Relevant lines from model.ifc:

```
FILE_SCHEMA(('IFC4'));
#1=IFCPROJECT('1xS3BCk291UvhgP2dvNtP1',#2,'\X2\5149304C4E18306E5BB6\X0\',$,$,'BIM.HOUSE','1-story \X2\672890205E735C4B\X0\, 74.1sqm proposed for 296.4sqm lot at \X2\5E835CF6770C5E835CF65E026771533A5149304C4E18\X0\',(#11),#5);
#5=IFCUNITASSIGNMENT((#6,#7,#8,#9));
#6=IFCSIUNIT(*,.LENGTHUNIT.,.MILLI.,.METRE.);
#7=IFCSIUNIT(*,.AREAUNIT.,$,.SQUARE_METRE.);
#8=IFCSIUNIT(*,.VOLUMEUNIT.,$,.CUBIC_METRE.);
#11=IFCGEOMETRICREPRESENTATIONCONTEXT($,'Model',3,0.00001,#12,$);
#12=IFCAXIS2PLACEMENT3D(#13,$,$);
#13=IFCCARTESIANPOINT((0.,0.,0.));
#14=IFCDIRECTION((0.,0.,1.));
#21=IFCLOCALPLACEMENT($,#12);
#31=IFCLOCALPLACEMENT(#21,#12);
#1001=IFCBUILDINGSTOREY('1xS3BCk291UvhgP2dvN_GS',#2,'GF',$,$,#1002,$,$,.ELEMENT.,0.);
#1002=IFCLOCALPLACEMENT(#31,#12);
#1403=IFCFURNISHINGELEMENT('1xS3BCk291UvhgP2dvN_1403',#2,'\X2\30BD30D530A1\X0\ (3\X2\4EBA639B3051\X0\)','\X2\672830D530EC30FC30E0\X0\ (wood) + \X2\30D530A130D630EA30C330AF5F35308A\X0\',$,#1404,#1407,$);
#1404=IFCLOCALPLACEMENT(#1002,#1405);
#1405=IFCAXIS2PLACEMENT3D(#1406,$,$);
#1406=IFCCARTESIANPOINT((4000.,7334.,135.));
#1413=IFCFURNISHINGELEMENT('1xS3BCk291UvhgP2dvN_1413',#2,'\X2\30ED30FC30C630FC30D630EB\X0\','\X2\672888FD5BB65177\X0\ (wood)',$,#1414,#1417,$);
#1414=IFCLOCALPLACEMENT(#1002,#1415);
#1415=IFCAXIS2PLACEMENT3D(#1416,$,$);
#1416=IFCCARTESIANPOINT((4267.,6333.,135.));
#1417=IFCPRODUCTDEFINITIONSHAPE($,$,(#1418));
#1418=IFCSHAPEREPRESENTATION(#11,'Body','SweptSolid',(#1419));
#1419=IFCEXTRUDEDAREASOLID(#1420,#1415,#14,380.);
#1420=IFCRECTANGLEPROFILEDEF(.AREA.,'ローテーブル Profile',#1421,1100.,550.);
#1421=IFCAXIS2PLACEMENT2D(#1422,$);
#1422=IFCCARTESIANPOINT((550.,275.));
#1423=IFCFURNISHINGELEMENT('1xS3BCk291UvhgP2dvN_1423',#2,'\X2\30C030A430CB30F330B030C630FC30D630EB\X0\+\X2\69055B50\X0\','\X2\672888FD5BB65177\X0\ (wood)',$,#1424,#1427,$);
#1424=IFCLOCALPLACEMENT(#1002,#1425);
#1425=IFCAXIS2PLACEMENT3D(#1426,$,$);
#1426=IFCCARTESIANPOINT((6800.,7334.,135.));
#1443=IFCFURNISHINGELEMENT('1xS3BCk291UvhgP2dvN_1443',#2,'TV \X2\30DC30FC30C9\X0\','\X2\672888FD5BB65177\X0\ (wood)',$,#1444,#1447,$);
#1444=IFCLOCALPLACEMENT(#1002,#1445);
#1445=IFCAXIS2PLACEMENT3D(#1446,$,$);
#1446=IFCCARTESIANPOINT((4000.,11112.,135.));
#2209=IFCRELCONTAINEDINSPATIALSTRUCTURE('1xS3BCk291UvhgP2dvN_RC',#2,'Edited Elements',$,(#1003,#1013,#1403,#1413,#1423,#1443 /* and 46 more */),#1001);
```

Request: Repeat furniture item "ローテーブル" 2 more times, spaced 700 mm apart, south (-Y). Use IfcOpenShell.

```python
import numpy as np
import ifcopenshell
import ifcopenshell.api.geometry
import ifcopenshell.api.root
import ifcopenshell.util.element
import ifcopenshell.util.placement
import ifcopenshell.util.unit

model = ifcopenshell.open("model.ifc")
unit_scale = ifcopenshell.util.unit.calculate_unit_scale(model)


def reuse_history(source, copy):
    """copy_class also copies each property set's owner history, people and application; keep the originals."""
    for rel in copy.IsDefinedBy:
        if rel.is_a("IfcRelDefinesByProperties") and (history := rel.RelatingPropertyDefinition.OwnerHistory):
            rel.RelatingPropertyDefinition.OwnerHistory = source.OwnerHistory
            ifcopenshell.util.element.remove_deep2(model, history)


source = model.by_id(1413)
base = ifcopenshell.util.placement.get_local_placement(source.ObjectPlacement)
step = np.array([0.0, -1.0, 0.0]) * 0.7 / unit_scale

for i in range(1, 3):
    copy = ifcopenshell.api.root.copy_class(model, product=source)
    copy.Representation = ifcopenshell.util.element.copy_deep(
        model, source.Representation, exclude=["IfcGeometricRepresentationContext", "IfcRepresentationMap"]
    )
    reuse_history(source, copy)
    matrix = base.copy()
    matrix[:3, 3] += i * step
    print("added at", matrix[:3, 3].round(3) + 0.0)
    ifcopenshell.api.geometry.edit_object_placement(model, product=copy, matrix=matrix, is_si=False)

model.write("model_v2.ifc")
```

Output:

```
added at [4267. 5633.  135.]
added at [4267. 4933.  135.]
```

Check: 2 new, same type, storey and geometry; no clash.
